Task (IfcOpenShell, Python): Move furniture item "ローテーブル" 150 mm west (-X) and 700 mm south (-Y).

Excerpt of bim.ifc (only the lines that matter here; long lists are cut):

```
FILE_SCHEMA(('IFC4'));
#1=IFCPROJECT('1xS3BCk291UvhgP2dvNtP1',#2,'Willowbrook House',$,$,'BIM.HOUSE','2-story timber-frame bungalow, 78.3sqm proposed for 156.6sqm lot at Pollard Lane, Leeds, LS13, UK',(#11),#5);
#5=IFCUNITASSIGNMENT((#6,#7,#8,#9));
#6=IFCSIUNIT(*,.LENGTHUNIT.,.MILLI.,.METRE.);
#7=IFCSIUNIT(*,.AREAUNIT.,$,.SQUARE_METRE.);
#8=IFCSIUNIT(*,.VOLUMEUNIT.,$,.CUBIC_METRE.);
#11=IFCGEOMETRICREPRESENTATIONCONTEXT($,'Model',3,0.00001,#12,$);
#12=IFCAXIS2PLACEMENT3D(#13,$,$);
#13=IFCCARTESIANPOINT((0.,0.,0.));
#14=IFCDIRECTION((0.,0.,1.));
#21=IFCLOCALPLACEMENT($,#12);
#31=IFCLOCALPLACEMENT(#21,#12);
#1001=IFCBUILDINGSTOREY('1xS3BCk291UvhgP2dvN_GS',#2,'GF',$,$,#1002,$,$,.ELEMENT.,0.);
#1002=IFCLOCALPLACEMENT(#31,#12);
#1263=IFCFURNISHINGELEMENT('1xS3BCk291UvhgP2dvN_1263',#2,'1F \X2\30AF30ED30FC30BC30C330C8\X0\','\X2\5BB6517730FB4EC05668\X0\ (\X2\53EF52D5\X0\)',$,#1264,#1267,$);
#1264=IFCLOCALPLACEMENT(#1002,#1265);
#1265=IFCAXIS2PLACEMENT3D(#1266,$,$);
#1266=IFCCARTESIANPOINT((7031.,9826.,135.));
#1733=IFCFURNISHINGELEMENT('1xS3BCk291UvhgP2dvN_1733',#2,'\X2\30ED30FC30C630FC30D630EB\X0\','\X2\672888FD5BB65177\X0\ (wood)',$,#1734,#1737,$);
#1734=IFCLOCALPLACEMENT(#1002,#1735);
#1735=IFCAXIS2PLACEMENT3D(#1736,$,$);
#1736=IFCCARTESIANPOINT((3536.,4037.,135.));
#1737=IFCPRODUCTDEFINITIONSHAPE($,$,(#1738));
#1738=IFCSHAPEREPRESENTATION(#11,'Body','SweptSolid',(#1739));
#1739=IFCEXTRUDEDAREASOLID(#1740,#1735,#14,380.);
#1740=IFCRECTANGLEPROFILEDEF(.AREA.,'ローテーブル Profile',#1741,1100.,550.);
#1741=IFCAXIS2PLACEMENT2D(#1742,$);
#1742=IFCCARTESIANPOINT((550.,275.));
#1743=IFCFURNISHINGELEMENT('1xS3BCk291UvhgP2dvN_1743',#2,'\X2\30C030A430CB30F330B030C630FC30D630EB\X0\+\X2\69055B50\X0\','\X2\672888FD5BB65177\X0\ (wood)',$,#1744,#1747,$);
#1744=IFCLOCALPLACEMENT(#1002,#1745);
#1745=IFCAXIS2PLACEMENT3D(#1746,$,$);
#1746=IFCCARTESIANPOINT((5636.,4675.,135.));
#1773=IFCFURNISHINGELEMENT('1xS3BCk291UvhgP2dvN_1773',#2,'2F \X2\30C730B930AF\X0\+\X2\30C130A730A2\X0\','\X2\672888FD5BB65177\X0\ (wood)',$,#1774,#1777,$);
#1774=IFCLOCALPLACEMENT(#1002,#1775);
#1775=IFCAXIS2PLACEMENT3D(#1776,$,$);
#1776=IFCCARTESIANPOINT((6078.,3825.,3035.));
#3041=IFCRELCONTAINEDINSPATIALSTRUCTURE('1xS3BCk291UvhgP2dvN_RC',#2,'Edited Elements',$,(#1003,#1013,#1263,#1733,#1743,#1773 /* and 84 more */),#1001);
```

```python
import ifcopenshell
import ifcopenshell.api.geometry
import ifcopenshell.util.placement
import ifcopenshell.util.unit

model = ifcopenshell.open("bim.ifc")
unit_scale = ifcopenshell.util.unit.calculate_unit_scale(model)

item = model.by_guid("1xS3BCk291UvhgP2dvN_1733")
matrix = ifcopenshell.util.placement.get_local_placement(item.ObjectPlacement)
matrix[0, 3] -= 0.15 / unit_scale
matrix[1, 3] -= 0.7 / unit_scale
ifcopenshell.api.geometry.edit_object_placement(model, product=item, matrix=matrix, is_si=False)

print(ifcopenshell.util.placement.get_local_placement(item.ObjectPlacement).round(3) + 0.0)

model.write("bim_updated.ifc")
```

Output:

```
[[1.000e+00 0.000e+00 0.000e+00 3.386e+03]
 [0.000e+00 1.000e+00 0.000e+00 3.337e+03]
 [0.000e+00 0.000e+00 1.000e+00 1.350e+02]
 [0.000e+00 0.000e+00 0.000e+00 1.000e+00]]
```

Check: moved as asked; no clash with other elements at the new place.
